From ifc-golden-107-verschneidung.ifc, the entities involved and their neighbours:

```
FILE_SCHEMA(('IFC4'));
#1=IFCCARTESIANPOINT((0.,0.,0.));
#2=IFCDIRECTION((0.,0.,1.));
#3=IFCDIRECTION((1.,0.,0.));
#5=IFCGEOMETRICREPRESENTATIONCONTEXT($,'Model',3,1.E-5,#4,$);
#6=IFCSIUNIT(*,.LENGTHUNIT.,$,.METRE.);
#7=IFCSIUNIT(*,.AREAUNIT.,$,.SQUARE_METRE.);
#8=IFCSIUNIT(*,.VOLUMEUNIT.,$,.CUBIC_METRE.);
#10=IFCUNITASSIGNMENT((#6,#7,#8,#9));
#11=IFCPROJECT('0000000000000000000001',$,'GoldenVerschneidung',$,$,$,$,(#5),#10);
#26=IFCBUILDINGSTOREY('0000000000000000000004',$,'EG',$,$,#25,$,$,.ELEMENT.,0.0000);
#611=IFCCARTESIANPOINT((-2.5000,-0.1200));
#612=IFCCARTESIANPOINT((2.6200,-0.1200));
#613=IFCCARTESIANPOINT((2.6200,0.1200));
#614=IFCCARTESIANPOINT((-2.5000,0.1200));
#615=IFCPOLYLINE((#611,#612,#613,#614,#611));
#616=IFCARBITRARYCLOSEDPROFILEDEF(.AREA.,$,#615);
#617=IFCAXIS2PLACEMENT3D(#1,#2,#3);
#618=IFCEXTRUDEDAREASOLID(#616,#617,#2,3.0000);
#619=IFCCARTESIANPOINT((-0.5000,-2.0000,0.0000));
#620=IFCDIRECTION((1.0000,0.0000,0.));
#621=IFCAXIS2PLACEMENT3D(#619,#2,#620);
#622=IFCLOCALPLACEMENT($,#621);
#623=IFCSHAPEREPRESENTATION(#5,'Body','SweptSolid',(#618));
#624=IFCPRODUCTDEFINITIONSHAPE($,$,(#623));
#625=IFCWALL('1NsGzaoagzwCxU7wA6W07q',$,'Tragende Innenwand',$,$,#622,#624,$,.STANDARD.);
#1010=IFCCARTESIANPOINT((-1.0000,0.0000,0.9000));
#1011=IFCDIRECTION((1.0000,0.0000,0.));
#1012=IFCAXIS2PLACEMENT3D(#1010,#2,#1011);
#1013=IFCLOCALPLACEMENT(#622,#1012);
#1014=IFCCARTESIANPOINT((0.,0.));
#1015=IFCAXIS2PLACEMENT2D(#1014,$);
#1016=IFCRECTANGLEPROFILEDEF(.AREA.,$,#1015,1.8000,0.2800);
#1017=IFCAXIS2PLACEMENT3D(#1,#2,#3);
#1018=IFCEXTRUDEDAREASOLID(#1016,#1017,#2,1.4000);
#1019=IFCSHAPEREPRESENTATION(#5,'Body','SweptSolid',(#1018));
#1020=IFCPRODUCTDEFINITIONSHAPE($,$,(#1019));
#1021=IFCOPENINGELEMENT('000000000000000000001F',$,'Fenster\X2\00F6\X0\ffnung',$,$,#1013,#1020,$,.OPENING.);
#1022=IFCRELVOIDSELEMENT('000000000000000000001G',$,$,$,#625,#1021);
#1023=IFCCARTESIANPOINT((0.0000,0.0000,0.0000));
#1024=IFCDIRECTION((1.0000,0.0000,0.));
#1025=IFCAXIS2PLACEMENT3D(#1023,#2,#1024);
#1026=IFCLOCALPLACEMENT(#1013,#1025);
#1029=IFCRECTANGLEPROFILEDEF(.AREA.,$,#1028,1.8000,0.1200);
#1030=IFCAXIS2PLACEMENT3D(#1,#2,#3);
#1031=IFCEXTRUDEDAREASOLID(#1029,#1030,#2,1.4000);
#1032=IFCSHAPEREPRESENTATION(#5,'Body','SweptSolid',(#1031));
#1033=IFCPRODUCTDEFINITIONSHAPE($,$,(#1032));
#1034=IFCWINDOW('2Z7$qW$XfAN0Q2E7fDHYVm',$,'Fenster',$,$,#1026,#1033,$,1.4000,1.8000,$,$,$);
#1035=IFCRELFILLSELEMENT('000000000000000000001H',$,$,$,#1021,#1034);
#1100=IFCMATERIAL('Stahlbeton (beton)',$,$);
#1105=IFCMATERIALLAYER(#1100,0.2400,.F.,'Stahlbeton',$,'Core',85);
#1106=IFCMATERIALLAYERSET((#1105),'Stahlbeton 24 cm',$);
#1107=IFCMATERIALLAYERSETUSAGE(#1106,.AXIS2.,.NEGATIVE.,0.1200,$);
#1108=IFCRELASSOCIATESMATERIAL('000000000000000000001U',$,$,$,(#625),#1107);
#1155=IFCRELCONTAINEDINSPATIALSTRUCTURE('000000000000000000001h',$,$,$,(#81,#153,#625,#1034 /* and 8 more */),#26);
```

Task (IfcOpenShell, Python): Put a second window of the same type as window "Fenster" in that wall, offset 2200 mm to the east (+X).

```python
import ifcopenshell
import ifcopenshell.api.feature
import ifcopenshell.api.geometry
import ifcopenshell.api.root
import ifcopenshell.geom
import ifcopenshell.util.element
import ifcopenshell.util.placement
import ifcopenshell.util.shape
import ifcopenshell.util.unit

model = ifcopenshell.open("ifc-golden-107-verschneidung.ifc")
unit_scale = ifcopenshell.util.unit.calculate_unit_scale(model)
settings = ifcopenshell.geom.settings()


def volume(element):
    """Net volume in cubic metres, openings subtracted."""
    shape = ifcopenshell.geom.create_shape(settings, element)
    return ifcopenshell.util.shape.get_volume(shape.geometry)


window = model.by_guid("2Z7$qW$XfAN0Q2E7fDHYVm")
opening = window.FillsVoids[0].RelatingOpeningElement
wall = opening.VoidsElements[0].RelatingBuildingElement
before = volume(wall)
shift = ifcopenshell.util.placement.get_local_placement(wall.ObjectPlacement)[:3, 0] * 2.2 / unit_scale

# copy_class copies the void relationship, type, container and properties, but no geometry.
new_opening = ifcopenshell.api.root.copy_class(model, product=opening)
new_opening.Representation = ifcopenshell.util.element.copy_deep(
    model, opening.Representation, exclude=["IfcGeometricRepresentationContext", "IfcRepresentationMap"]
)
new_window = ifcopenshell.api.root.copy_class(model, product=window)
new_window.Representation = ifcopenshell.util.element.copy_deep(
    model, window.Representation, exclude=["IfcGeometricRepresentationContext", "IfcRepresentationMap"]
)
ifcopenshell.api.feature.add_filling(model, opening=new_opening, element=new_window)

for old, new in ((opening, new_opening), (window, new_window)):
    matrix = ifcopenshell.util.placement.get_local_placement(old.ObjectPlacement)
    matrix[:3, 3] += shift
    ifcopenshell.api.geometry.edit_object_placement(model, product=new, matrix=matrix, is_si=False)

after = volume(wall)

print(f"wall volume {before:.3f} -> {after:.3f} m3")

model.write("ifc-golden-107-verschneidung-out.ifc")
```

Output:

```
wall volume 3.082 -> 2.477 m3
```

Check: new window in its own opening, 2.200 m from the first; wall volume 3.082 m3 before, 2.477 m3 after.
